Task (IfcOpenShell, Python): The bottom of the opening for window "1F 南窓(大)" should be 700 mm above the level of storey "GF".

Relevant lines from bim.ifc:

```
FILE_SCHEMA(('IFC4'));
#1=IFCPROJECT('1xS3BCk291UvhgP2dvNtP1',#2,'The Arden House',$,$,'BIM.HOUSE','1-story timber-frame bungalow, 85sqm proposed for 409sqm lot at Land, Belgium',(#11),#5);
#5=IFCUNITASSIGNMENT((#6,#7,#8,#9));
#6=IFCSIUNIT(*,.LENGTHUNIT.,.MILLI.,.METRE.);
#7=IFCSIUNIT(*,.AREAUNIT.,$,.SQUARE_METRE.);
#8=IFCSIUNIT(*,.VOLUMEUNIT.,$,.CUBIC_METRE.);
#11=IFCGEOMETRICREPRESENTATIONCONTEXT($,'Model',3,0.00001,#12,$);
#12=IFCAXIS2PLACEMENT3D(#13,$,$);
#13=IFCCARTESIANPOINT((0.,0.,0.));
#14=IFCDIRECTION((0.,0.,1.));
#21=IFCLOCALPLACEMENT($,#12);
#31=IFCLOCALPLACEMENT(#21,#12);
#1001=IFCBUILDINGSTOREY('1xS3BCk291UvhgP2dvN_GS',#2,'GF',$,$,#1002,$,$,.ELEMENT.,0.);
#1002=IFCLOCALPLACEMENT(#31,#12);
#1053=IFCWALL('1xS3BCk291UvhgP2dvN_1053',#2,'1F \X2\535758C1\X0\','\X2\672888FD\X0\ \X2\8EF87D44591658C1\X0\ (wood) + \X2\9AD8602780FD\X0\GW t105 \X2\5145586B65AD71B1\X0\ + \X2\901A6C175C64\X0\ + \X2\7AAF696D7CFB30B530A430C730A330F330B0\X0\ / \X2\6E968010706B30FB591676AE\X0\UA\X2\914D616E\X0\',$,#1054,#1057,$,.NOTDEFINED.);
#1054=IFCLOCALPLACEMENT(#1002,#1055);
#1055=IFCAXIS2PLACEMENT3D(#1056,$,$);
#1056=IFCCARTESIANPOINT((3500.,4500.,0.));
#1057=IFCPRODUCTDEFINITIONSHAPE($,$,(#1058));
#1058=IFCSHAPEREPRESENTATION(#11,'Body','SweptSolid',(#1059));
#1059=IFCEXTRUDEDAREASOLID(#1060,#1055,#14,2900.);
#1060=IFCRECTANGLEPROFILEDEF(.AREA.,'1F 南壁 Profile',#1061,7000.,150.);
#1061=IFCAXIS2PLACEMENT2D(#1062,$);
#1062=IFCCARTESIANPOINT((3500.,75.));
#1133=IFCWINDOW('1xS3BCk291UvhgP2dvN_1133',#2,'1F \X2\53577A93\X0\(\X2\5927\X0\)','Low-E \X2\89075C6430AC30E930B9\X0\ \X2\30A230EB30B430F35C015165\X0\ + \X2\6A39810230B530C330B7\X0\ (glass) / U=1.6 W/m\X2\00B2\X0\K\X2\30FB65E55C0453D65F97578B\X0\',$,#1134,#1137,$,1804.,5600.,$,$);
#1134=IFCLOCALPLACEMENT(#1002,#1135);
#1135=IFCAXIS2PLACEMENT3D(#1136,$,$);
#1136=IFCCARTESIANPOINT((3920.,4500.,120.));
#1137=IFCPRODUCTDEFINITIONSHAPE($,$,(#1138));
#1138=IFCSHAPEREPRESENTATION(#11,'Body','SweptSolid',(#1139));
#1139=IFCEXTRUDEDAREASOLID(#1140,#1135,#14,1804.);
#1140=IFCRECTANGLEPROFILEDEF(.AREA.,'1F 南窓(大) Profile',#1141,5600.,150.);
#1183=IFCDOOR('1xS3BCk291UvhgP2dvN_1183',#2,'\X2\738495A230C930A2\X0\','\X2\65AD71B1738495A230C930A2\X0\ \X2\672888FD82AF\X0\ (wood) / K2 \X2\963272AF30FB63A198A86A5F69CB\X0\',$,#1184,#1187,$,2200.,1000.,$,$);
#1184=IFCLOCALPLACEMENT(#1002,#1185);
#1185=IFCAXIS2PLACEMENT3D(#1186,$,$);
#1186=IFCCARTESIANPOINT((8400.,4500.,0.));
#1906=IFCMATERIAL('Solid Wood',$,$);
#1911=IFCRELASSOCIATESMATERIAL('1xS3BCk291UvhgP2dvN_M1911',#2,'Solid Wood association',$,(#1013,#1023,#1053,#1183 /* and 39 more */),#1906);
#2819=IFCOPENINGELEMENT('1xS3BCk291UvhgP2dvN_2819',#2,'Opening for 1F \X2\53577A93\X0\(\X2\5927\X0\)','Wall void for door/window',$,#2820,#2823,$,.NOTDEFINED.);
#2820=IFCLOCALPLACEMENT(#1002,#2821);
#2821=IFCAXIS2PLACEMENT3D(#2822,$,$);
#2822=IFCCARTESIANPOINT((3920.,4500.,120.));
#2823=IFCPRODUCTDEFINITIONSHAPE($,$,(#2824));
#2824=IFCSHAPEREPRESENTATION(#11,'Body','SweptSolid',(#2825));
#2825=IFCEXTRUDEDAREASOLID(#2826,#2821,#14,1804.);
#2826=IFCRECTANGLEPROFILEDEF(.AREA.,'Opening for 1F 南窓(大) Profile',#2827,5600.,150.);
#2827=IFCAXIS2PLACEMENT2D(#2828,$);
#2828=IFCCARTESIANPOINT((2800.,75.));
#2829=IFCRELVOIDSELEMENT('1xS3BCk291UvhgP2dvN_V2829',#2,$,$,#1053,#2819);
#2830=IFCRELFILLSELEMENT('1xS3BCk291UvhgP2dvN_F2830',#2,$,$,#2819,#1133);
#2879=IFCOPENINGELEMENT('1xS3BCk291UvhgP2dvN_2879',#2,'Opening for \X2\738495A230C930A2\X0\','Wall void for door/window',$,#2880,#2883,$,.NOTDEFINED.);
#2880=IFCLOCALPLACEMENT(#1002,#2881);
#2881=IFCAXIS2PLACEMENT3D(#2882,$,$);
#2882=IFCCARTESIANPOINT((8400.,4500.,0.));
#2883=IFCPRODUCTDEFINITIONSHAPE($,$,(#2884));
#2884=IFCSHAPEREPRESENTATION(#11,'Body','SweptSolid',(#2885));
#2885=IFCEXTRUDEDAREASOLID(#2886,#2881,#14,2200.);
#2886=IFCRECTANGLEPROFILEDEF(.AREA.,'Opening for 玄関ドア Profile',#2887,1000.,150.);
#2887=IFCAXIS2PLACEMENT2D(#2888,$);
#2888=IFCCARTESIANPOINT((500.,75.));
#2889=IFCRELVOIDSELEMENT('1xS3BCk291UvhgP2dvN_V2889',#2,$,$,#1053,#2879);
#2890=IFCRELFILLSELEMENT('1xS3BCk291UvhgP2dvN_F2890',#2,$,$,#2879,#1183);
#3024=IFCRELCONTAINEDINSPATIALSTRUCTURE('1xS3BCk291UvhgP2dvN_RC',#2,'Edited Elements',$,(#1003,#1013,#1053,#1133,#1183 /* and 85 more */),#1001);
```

```python
import numpy as np
import ifcopenshell
import ifcopenshell.api.geometry
import ifcopenshell.geom
import ifcopenshell.util.element
import ifcopenshell.util.placement
import ifcopenshell.util.shape
import ifcopenshell.util.unit

model = ifcopenshell.open("bim.ifc")
unit_scale = ifcopenshell.util.unit.calculate_unit_scale(model)

window = model.by_guid("1xS3BCk291UvhgP2dvN_1133")
opening = window.FillsVoids[0].RelatingOpeningElement
storey = ifcopenshell.util.element.get_container(window, ifc_class="IfcBuildingStorey")
level = ifcopenshell.util.placement.get_local_placement(storey.ObjectPlacement)[2, 3]

# The opening's origin need not be at the sill, so measure its lowest point.
shape = ifcopenshell.geom.create_shape(ifcopenshell.geom.settings(), opening)
bottom = ifcopenshell.util.shape.get_shape_bottom_elevation(shape, shape.geometry) / unit_scale
dz = level + 700.0 - bottom

shift = np.array([0.0, 0.0, dz])
# The window is not placed relative to its opening, so move both.
for product in (opening, window):
    matrix = ifcopenshell.util.placement.get_local_placement(product.ObjectPlacement)
    matrix[:3, 3] += shift
    ifcopenshell.api.geometry.edit_object_placement(model, product=product, matrix=matrix, is_si=False)

print(f"moved by {dz * unit_scale:+.3f} m")

model.write("bim-out.ifc")
```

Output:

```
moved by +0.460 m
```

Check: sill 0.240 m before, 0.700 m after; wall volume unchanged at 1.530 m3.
